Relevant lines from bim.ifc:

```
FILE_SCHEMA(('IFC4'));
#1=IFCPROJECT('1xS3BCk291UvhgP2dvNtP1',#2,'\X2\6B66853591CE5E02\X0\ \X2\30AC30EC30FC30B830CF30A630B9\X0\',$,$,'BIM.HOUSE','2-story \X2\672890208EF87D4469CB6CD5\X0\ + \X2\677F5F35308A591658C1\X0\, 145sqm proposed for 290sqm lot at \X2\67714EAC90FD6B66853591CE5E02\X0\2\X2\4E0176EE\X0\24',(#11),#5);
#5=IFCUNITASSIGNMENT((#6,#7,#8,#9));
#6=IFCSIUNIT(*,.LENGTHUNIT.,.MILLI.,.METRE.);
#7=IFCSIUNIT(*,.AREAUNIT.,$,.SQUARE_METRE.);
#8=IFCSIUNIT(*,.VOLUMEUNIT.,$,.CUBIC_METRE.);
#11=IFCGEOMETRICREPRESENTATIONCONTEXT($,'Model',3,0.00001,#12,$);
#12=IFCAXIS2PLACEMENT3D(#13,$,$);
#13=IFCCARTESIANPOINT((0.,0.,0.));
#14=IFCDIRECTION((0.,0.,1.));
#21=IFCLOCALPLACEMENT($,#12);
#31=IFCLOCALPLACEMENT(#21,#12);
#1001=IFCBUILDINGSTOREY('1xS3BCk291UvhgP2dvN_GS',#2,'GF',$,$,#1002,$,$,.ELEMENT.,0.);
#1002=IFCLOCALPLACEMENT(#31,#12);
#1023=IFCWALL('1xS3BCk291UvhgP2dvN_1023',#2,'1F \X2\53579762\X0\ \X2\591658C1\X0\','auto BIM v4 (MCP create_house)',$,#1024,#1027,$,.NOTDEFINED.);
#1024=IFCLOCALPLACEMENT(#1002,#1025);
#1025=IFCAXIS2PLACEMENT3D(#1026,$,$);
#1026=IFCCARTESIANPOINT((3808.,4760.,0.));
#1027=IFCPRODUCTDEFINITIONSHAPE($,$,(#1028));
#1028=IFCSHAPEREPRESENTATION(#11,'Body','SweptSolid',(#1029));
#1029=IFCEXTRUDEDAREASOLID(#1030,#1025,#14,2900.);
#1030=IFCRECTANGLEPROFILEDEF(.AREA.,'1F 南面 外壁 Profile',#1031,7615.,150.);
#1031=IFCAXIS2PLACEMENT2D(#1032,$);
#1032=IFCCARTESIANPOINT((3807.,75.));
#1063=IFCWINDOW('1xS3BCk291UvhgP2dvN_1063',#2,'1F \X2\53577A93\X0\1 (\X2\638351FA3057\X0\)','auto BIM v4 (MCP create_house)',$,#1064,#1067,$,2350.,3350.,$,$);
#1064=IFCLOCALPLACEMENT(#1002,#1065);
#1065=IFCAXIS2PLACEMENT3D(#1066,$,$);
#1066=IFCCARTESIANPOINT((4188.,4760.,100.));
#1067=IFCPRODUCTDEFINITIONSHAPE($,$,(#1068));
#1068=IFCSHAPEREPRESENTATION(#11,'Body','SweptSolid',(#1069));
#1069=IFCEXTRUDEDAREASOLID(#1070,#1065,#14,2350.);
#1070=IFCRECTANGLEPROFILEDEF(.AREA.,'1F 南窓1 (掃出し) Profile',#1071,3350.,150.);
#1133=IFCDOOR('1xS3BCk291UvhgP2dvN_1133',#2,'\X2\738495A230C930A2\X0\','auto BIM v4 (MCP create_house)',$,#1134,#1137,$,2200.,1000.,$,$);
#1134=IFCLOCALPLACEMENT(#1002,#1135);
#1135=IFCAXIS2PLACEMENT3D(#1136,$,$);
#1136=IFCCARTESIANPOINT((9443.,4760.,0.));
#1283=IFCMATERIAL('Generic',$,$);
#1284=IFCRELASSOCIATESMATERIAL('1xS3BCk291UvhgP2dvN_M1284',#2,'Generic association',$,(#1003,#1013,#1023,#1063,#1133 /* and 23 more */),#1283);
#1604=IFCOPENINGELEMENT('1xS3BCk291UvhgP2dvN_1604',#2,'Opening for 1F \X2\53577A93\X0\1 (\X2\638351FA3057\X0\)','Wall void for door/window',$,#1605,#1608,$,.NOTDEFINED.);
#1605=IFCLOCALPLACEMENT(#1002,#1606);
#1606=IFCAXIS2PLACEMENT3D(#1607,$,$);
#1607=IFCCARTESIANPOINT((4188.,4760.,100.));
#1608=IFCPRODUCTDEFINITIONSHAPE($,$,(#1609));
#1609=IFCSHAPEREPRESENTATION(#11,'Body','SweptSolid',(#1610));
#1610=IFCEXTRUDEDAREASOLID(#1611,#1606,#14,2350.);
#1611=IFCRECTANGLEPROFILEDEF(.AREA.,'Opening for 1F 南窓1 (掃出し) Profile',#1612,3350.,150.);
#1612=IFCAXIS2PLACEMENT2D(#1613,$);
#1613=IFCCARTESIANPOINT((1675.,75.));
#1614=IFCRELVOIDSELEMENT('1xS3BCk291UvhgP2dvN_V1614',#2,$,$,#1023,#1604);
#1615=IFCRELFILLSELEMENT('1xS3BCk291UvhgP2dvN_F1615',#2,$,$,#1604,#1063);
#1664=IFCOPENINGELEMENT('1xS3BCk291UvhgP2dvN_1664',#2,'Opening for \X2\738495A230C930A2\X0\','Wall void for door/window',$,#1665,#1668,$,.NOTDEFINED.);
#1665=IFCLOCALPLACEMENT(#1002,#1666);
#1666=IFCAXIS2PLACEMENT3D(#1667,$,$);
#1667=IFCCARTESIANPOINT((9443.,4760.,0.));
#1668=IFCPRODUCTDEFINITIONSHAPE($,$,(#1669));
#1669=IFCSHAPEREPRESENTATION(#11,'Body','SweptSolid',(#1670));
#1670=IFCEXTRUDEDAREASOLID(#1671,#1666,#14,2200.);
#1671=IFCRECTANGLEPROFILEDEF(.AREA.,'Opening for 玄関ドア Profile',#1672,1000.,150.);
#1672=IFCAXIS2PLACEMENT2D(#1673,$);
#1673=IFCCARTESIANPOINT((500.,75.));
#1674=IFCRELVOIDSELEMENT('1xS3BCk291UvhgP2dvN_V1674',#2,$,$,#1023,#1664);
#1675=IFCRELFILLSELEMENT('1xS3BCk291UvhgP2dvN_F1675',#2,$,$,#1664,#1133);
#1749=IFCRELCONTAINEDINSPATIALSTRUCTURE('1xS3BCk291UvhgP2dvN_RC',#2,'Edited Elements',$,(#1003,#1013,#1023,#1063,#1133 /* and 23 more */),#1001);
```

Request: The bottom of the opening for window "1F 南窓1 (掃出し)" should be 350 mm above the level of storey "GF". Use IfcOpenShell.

```python
import numpy as np
import ifcopenshell
import ifcopenshell.api.geometry
import ifcopenshell.geom
import ifcopenshell.util.element
import ifcopenshell.util.placement
import ifcopenshell.util.shape
import ifcopenshell.util.unit

model = ifcopenshell.open("bim.ifc")
unit_scale = ifcopenshell.util.unit.calculate_unit_scale(model)

window = model.by_guid("1xS3BCk291UvhgP2dvN_1063")
opening = window.FillsVoids[0].RelatingOpeningElement
storey = ifcopenshell.util.element.get_container(window, ifc_class="IfcBuildingStorey")
level = ifcopenshell.util.placement.get_local_placement(storey.ObjectPlacement)[2, 3]

# The opening's origin need not be at the sill, so measure its lowest point.
shape = ifcopenshell.geom.create_shape(ifcopenshell.geom.settings(), opening)
bottom = ifcopenshell.util.shape.get_shape_bottom_elevation(shape, shape.geometry) / unit_scale
dz = level + 350.0 - bottom

shift = np.array([0.0, 0.0, dz])
# The window is not placed relative to its opening, so move both.
for product in (opening, window):
    matrix = ifcopenshell.util.placement.get_local_placement(product.ObjectPlacement)
    matrix[:3, 3] += shift
    ifcopenshell.api.geometry.edit_object_placement(model, product=product, matrix=matrix, is_si=False)

print(f"moved by {dz * unit_scale:+.3f} m")

model.write("bim_v2.ifc")
```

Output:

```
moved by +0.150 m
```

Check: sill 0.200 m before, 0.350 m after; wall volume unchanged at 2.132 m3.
